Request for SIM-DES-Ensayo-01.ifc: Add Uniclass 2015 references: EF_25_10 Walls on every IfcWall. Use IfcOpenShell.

First a look at what the model holds.

```python
import ifcopenshell

model = ifcopenshell.open("SIM-DES-Ensayo-01.ifc")
print(model.schema)
print("classifications:", [c.Name for c in model.by_type("IfcClassification")])
for ifc_class in ("IfcDoor", "IfcRoof", "IfcStair", "IfcWall", "IfcWindow"):
    print(ifc_class, len(model.by_type(ifc_class)))
```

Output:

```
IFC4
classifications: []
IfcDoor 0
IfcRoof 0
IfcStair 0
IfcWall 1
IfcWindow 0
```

```python
import ifcopenshell
import ifcopenshell.api.classification

model = ifcopenshell.open("SIM-DES-Ensayo-01.ifc")

system = ifcopenshell.api.classification.add_classification(model, classification="Uniclass 2015")

codes = {
    "IfcWall": ("EF_25_10", "Walls"),
}
for ifc_class, (code, name) in codes.items():
    products = model.by_type(ifc_class)
    ifcopenshell.api.classification.add_reference(
        model, products=products, classification=system, identification=code, name=name
    )
    print(code, len(products))

model.write("SIM-DES-Ensayo-01_updated.ifc")
```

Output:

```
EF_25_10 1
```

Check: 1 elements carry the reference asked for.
